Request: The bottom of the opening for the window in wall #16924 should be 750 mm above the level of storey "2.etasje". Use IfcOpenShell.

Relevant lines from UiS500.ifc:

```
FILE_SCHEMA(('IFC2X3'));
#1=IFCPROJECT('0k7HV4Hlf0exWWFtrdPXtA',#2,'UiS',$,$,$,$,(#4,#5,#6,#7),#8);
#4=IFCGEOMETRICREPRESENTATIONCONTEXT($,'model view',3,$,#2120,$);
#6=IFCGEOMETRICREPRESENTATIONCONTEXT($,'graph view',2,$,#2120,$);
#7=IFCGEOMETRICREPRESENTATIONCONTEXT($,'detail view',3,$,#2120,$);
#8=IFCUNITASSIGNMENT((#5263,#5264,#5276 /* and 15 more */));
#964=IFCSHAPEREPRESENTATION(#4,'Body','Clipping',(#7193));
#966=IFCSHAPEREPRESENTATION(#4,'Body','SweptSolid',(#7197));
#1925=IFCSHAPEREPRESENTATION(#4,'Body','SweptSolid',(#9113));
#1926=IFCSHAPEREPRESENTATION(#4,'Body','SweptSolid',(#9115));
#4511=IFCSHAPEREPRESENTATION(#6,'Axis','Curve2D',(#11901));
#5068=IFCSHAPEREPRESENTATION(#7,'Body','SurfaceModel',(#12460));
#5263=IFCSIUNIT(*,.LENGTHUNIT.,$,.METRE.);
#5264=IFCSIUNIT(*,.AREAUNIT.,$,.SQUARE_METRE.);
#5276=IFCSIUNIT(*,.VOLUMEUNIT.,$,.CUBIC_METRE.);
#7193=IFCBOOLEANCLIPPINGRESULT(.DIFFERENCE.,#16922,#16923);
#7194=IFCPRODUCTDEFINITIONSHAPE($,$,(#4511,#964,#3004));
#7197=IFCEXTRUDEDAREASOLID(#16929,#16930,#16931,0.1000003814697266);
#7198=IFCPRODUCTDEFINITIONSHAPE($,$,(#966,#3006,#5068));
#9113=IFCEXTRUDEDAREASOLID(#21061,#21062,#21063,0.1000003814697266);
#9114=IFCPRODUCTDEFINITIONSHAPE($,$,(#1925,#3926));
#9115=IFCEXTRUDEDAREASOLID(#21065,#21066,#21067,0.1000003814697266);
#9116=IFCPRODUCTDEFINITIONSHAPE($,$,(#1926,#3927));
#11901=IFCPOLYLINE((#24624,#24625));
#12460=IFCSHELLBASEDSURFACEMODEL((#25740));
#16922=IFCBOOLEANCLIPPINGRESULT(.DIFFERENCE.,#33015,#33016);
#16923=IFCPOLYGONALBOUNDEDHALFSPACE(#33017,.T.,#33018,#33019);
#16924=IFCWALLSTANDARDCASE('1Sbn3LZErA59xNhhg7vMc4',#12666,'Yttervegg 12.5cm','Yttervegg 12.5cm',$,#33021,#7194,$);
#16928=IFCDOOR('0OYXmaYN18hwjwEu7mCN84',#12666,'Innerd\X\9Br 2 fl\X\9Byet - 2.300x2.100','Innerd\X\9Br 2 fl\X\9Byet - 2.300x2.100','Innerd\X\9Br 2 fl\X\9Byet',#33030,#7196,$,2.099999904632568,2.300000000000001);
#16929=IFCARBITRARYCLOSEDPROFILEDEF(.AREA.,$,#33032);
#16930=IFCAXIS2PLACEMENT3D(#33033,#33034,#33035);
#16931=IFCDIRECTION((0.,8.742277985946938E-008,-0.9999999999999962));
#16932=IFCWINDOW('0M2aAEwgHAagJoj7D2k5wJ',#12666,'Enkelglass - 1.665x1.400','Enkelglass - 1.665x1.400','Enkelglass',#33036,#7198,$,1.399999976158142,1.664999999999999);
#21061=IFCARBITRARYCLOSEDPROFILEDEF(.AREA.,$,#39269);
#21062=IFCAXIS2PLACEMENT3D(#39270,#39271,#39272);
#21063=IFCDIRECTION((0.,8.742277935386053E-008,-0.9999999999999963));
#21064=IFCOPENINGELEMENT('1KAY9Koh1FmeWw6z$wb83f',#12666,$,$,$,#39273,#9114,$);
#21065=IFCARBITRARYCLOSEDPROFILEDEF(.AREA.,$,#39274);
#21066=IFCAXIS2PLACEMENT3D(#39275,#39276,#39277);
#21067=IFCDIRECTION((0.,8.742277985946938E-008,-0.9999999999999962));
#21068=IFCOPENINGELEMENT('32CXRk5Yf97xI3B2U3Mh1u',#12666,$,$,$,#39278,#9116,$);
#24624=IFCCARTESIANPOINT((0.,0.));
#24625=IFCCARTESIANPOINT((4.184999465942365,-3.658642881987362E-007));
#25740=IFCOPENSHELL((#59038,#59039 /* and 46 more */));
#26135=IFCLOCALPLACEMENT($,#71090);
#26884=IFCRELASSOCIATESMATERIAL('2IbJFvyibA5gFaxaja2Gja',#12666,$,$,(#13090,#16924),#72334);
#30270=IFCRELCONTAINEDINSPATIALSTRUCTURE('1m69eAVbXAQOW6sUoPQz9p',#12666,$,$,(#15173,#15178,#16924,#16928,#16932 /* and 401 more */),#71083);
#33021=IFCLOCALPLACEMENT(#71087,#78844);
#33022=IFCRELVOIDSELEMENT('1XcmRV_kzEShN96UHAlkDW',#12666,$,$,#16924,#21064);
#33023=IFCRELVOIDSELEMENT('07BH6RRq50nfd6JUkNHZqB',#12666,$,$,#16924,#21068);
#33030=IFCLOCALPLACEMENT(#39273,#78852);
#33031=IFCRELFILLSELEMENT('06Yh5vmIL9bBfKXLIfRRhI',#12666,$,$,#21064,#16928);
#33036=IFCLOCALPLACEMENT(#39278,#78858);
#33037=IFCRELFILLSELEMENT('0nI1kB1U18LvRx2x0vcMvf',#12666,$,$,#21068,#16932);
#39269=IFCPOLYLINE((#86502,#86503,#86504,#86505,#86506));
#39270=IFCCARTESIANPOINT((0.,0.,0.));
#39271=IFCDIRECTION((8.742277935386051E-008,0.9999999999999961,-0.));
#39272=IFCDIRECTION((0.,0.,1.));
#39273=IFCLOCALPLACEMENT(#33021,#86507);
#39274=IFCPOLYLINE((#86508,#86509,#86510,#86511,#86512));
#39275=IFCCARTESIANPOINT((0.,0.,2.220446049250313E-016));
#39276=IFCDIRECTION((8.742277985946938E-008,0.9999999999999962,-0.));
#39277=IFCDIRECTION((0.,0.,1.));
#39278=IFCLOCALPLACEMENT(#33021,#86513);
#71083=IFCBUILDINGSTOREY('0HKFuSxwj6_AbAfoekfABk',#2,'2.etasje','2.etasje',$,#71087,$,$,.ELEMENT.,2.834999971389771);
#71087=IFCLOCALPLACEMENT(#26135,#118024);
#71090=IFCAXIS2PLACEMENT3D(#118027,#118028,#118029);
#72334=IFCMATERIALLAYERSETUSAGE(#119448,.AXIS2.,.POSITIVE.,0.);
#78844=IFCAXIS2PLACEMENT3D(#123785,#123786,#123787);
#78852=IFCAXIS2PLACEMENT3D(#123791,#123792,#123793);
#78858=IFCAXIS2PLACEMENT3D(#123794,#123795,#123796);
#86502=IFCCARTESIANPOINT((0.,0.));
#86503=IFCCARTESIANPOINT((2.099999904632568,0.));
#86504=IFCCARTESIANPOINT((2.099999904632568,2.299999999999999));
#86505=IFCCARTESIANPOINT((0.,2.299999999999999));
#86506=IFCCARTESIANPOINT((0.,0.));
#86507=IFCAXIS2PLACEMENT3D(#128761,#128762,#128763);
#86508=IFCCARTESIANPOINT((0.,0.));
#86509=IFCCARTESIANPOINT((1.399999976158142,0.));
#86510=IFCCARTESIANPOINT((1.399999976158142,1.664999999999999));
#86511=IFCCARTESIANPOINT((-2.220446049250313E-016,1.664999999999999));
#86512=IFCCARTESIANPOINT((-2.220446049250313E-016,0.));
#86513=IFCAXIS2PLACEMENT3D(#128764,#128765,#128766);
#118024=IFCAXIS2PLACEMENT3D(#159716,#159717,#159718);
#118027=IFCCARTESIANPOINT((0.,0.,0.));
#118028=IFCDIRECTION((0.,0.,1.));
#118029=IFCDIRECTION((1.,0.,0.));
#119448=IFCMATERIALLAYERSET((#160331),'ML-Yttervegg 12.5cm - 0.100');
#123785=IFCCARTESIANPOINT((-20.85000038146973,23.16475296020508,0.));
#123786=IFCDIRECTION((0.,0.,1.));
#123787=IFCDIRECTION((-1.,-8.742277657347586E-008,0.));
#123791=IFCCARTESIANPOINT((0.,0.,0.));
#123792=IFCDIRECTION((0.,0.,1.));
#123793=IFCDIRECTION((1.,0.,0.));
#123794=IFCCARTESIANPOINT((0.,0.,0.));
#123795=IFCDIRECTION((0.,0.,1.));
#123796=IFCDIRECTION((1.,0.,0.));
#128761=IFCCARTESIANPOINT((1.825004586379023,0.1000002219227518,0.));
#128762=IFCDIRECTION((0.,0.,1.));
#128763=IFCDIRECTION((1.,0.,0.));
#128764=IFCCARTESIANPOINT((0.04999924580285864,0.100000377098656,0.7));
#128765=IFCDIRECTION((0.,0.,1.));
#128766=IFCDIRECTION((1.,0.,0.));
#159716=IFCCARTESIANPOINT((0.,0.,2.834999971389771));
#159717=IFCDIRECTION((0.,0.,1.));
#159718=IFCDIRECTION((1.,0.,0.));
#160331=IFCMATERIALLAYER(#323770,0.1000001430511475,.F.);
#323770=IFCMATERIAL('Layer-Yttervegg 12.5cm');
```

```python
import numpy as np
import ifcopenshell
import ifcopenshell.api.geometry
import ifcopenshell.geom
import ifcopenshell.util.element
import ifcopenshell.util.placement
import ifcopenshell.util.shape
import ifcopenshell.util.unit

model = ifcopenshell.open("UiS500.ifc")
unit_scale = ifcopenshell.util.unit.calculate_unit_scale(model)

window = model.by_guid("0M2aAEwgHAagJoj7D2k5wJ")
opening = window.FillsVoids[0].RelatingOpeningElement
storey = ifcopenshell.util.element.get_container(window, ifc_class="IfcBuildingStorey")
level = ifcopenshell.util.placement.get_local_placement(storey.ObjectPlacement)[2, 3]

# The opening's origin need not be at the sill, so measure its lowest point.
shape = ifcopenshell.geom.create_shape(ifcopenshell.geom.settings(), opening)
bottom = ifcopenshell.util.shape.get_shape_bottom_elevation(shape, shape.geometry) / unit_scale
dz = level + 0.75 / unit_scale - bottom

shift = np.array([0.0, 0.0, dz])
# The window is placed relative to its opening, so it follows when the opening moves.
matrix = ifcopenshell.util.placement.get_local_placement(opening.ObjectPlacement)
matrix[:3, 3] += shift
ifcopenshell.api.geometry.edit_object_placement(
    model, product=opening, matrix=matrix, is_si=False, should_transform_children=True
)

print(f"moved by {dz * unit_scale:+.3f} m")

model.write("UiS500_v2.ifc")
```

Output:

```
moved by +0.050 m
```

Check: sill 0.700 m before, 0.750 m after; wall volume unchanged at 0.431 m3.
